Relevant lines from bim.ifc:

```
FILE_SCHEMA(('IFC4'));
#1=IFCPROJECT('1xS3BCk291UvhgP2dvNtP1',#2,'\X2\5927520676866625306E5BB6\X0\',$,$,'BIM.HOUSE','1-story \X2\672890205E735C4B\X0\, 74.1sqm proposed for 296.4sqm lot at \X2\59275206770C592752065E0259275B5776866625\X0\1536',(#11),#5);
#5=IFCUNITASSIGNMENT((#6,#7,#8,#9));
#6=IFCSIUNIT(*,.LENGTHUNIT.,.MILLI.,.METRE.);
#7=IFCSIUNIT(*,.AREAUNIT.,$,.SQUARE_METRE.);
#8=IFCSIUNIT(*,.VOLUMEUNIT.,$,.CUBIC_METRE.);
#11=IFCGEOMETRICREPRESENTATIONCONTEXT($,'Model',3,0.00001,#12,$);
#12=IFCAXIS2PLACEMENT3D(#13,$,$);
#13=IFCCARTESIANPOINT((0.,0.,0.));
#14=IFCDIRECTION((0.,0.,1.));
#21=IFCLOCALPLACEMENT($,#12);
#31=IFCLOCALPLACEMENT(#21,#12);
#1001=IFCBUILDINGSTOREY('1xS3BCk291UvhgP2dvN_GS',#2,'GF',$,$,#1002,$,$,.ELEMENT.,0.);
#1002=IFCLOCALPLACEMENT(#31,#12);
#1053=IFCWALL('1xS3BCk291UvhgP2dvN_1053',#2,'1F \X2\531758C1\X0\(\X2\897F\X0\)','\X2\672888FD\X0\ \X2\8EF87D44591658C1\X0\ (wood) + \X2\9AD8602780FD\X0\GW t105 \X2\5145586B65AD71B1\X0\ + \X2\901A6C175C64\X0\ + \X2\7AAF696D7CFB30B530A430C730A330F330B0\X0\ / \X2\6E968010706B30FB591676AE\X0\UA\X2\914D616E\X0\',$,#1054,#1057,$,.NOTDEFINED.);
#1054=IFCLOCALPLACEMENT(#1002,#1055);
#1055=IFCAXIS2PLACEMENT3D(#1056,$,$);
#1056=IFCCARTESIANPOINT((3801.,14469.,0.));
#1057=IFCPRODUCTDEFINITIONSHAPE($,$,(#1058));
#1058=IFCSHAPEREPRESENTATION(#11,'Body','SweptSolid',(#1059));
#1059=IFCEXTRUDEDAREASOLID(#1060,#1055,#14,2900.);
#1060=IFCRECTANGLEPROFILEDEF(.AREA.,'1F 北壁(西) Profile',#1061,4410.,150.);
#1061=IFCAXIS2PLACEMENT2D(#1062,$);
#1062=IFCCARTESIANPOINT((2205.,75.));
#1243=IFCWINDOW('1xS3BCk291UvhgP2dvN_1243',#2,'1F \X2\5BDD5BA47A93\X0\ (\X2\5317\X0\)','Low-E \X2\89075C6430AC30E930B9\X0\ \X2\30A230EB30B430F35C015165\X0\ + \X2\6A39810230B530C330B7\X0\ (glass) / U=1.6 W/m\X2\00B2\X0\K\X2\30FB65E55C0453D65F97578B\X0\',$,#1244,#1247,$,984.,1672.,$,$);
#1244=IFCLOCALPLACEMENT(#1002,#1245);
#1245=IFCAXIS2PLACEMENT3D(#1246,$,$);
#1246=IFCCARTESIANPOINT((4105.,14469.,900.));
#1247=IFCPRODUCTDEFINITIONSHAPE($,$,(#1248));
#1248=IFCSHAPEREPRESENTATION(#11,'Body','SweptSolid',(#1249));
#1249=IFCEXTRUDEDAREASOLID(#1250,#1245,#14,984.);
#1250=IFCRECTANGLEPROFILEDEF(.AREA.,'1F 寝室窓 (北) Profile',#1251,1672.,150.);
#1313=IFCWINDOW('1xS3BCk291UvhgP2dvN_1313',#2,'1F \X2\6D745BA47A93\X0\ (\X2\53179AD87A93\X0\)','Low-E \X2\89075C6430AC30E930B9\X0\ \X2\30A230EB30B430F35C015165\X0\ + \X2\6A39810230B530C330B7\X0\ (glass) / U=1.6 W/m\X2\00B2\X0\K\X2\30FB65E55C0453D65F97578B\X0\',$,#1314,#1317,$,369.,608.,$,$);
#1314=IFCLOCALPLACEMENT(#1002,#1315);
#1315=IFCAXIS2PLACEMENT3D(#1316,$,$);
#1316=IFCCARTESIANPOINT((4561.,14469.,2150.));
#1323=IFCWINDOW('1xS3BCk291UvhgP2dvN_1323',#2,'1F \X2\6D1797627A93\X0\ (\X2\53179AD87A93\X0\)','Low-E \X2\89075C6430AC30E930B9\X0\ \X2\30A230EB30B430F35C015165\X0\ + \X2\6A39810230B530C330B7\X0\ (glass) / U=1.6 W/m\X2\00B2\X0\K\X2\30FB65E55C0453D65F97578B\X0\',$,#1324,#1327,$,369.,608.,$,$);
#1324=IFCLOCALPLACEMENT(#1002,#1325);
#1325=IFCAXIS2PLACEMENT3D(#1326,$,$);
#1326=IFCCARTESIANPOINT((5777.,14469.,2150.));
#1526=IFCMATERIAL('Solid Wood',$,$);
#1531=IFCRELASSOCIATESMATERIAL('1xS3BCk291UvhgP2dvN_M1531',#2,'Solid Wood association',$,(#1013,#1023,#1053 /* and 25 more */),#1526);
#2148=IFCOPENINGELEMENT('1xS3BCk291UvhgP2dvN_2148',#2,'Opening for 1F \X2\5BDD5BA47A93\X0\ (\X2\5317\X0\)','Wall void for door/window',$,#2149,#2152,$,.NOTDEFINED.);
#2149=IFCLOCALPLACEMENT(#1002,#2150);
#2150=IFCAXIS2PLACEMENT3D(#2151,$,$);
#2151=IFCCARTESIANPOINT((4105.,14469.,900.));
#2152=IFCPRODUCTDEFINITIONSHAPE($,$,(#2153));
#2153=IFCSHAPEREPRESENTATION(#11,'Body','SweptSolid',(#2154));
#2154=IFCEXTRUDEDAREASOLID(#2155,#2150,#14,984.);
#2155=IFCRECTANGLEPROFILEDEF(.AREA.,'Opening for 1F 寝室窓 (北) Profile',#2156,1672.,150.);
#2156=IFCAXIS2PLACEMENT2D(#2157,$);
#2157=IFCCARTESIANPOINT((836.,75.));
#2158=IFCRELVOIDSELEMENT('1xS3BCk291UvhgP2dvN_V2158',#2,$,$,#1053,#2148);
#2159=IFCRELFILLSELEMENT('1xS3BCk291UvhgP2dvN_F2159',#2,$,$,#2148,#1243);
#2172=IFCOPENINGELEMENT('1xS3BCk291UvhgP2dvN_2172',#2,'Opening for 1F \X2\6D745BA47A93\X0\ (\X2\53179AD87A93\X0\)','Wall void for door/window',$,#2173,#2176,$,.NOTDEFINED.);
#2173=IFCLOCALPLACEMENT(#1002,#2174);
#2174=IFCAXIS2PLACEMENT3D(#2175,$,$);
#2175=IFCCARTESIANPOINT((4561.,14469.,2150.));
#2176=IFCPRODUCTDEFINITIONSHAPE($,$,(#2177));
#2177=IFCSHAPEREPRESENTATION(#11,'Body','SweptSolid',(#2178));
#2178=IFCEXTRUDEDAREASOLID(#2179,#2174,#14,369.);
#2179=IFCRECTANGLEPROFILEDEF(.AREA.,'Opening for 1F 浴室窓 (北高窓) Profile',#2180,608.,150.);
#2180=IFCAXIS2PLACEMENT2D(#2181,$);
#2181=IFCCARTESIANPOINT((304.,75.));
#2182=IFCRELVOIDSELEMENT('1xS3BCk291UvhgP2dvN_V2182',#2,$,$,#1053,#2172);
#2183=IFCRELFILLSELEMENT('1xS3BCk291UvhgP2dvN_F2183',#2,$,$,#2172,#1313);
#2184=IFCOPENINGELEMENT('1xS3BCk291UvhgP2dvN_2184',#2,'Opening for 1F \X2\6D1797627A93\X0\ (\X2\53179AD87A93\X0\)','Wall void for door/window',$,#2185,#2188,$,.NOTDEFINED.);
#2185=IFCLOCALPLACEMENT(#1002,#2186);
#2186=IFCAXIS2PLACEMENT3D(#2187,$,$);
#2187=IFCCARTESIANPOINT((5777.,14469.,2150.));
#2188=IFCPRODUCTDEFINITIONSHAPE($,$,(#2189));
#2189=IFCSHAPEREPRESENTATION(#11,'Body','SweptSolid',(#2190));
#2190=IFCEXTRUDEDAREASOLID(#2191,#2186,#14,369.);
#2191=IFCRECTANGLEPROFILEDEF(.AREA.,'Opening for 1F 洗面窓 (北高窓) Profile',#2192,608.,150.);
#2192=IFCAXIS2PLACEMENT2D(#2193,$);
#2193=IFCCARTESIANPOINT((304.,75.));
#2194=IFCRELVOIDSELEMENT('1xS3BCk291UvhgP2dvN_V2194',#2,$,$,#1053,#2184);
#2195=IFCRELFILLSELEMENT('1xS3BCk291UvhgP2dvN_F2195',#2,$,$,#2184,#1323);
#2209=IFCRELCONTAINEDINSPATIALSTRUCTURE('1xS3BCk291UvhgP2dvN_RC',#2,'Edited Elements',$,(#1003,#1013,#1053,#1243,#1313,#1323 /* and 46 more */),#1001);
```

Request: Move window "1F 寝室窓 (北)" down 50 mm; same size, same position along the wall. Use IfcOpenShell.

```python
import numpy as np
import ifcopenshell
import ifcopenshell.api.geometry
import ifcopenshell.util.placement
import ifcopenshell.util.unit

model = ifcopenshell.open("bim.ifc")
unit_scale = ifcopenshell.util.unit.calculate_unit_scale(model)

window = model.by_guid("1xS3BCk291UvhgP2dvN_1243")
opening = window.FillsVoids[0].RelatingOpeningElement
dz = -50.0

shift = np.array([0.0, 0.0, dz])
# The window is not placed relative to its opening, so move both.
for product in (opening, window):
    matrix = ifcopenshell.util.placement.get_local_placement(product.ObjectPlacement)
    matrix[:3, 3] += shift
    ifcopenshell.api.geometry.edit_object_placement(model, product=product, matrix=matrix, is_si=False)

print(f"moved by {dz * unit_scale:+.3f} m")

model.write("bim_updated.ifc")
```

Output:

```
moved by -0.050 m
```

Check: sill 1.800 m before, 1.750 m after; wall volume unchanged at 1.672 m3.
